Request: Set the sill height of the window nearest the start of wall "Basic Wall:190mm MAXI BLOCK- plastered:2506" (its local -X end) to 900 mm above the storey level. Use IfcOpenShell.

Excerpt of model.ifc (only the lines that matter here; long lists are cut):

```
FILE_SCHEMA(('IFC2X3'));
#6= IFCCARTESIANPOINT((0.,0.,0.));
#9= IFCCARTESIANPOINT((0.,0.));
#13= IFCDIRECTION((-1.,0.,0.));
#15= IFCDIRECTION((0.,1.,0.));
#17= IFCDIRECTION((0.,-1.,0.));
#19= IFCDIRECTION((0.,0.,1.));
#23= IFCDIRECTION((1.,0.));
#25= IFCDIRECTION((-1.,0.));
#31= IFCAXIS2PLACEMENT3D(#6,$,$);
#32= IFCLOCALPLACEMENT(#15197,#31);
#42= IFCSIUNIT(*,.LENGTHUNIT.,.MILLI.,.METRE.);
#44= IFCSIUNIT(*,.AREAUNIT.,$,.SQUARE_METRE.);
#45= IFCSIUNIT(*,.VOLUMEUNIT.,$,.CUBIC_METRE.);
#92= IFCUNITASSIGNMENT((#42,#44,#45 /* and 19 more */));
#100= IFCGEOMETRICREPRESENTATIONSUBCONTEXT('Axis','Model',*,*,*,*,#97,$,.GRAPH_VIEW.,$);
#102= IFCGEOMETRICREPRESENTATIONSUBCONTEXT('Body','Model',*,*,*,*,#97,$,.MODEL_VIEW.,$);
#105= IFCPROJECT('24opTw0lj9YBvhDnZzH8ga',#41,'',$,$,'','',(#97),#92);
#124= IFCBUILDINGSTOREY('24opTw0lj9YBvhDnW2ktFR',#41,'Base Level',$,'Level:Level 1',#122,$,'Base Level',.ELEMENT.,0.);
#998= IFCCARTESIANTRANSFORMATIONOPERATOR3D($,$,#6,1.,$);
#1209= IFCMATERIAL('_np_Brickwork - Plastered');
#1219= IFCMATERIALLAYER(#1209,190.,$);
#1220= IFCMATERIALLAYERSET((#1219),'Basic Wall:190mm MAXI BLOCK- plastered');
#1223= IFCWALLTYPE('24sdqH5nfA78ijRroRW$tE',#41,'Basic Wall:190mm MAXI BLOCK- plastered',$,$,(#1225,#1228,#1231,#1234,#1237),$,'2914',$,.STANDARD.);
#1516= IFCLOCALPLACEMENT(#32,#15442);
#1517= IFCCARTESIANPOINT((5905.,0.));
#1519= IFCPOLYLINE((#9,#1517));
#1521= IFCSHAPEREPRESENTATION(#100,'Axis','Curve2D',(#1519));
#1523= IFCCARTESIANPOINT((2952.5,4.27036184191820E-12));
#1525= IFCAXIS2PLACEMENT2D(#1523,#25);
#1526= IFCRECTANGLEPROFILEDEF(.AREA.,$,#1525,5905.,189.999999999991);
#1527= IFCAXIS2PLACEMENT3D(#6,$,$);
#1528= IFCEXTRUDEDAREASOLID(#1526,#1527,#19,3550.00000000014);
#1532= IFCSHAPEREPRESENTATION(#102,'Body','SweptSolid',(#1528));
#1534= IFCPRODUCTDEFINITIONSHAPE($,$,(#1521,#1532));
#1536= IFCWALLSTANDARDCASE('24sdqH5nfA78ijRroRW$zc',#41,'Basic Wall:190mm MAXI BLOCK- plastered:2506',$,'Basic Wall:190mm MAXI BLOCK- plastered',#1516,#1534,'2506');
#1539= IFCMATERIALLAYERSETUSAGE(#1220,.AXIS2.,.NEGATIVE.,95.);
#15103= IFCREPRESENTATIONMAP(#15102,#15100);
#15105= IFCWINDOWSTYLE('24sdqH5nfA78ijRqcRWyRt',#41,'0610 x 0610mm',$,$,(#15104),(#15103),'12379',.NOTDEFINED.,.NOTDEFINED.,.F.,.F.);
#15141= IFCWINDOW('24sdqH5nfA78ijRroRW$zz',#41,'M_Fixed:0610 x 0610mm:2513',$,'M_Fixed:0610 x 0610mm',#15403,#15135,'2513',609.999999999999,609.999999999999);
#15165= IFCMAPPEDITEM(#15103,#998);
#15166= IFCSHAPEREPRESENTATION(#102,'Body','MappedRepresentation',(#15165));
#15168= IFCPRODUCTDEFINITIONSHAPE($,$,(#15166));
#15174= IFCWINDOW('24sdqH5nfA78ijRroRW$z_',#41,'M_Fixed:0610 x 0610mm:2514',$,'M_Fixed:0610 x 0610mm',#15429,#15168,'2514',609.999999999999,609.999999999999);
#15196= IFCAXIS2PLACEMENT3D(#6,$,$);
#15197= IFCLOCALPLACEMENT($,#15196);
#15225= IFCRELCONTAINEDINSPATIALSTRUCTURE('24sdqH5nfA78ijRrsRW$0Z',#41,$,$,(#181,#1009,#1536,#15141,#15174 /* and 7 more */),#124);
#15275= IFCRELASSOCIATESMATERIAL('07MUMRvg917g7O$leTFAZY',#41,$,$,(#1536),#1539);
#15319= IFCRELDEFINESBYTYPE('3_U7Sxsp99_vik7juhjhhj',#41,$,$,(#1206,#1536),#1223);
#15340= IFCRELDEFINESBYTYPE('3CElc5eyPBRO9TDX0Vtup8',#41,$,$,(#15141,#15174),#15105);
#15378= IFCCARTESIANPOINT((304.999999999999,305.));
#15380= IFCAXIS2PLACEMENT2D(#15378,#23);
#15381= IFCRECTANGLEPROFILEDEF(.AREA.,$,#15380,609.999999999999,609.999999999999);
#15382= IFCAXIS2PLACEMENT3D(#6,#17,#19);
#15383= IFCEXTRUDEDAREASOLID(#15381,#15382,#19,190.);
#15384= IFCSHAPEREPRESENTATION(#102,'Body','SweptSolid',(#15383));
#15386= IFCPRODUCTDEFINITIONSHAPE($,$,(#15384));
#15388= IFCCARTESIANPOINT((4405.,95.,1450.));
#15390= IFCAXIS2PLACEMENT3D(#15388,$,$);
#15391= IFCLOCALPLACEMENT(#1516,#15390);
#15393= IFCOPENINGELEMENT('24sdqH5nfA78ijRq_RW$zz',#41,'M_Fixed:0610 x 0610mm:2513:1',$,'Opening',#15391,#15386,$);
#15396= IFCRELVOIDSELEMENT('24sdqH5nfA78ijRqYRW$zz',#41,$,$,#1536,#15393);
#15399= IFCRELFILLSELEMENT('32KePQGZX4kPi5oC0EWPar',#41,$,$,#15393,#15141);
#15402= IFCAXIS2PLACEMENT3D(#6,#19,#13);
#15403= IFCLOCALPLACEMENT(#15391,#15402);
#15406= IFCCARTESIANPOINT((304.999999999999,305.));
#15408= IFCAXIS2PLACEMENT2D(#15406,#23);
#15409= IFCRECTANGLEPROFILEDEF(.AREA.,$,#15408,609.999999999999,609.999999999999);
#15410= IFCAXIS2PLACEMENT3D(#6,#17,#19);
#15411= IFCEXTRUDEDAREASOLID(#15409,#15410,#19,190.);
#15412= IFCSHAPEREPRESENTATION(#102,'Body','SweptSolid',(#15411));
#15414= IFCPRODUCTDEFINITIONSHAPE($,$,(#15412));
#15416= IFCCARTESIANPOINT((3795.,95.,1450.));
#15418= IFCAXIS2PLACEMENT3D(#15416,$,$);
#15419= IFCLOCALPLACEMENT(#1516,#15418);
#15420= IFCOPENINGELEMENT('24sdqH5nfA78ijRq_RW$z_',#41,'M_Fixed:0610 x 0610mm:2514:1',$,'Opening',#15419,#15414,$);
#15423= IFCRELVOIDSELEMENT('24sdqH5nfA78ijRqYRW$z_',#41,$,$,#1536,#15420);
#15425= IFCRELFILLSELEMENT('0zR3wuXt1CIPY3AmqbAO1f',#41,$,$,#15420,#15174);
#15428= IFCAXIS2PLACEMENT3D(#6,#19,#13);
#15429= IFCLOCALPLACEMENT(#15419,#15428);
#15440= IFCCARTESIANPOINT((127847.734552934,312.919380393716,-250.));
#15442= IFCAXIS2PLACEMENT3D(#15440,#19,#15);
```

```python
import numpy as np
import ifcopenshell
import ifcopenshell.api.geometry
import ifcopenshell.geom
import ifcopenshell.util.element
import ifcopenshell.util.placement
import ifcopenshell.util.shape
import ifcopenshell.util.unit

model = ifcopenshell.open("model.ifc")
unit_scale = ifcopenshell.util.unit.calculate_unit_scale(model)

window = model.by_guid("24sdqH5nfA78ijRroRW$z_")
opening = window.FillsVoids[0].RelatingOpeningElement
storey = ifcopenshell.util.element.get_container(window, ifc_class="IfcBuildingStorey")
level = ifcopenshell.util.placement.get_local_placement(storey.ObjectPlacement)[2, 3]

# The opening's origin need not be at the sill, so measure its lowest point.
shape = ifcopenshell.geom.create_shape(ifcopenshell.geom.settings(), opening)
bottom = ifcopenshell.util.shape.get_shape_bottom_elevation(shape, shape.geometry) / unit_scale
dz = level + 0.9 / unit_scale - bottom

shift = np.array([0.0, 0.0, dz])
# The window is placed relative to its opening, so it follows when the opening moves.
matrix = ifcopenshell.util.placement.get_local_placement(opening.ObjectPlacement)
matrix[:3, 3] += shift
ifcopenshell.api.geometry.edit_object_placement(
    model, product=opening, matrix=matrix, is_si=False, should_transform_children=True
)

print(f"moved by {dz * unit_scale:+.3f} m")

model.write("model_updated.ifc")
```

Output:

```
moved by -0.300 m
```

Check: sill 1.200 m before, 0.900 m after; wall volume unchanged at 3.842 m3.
